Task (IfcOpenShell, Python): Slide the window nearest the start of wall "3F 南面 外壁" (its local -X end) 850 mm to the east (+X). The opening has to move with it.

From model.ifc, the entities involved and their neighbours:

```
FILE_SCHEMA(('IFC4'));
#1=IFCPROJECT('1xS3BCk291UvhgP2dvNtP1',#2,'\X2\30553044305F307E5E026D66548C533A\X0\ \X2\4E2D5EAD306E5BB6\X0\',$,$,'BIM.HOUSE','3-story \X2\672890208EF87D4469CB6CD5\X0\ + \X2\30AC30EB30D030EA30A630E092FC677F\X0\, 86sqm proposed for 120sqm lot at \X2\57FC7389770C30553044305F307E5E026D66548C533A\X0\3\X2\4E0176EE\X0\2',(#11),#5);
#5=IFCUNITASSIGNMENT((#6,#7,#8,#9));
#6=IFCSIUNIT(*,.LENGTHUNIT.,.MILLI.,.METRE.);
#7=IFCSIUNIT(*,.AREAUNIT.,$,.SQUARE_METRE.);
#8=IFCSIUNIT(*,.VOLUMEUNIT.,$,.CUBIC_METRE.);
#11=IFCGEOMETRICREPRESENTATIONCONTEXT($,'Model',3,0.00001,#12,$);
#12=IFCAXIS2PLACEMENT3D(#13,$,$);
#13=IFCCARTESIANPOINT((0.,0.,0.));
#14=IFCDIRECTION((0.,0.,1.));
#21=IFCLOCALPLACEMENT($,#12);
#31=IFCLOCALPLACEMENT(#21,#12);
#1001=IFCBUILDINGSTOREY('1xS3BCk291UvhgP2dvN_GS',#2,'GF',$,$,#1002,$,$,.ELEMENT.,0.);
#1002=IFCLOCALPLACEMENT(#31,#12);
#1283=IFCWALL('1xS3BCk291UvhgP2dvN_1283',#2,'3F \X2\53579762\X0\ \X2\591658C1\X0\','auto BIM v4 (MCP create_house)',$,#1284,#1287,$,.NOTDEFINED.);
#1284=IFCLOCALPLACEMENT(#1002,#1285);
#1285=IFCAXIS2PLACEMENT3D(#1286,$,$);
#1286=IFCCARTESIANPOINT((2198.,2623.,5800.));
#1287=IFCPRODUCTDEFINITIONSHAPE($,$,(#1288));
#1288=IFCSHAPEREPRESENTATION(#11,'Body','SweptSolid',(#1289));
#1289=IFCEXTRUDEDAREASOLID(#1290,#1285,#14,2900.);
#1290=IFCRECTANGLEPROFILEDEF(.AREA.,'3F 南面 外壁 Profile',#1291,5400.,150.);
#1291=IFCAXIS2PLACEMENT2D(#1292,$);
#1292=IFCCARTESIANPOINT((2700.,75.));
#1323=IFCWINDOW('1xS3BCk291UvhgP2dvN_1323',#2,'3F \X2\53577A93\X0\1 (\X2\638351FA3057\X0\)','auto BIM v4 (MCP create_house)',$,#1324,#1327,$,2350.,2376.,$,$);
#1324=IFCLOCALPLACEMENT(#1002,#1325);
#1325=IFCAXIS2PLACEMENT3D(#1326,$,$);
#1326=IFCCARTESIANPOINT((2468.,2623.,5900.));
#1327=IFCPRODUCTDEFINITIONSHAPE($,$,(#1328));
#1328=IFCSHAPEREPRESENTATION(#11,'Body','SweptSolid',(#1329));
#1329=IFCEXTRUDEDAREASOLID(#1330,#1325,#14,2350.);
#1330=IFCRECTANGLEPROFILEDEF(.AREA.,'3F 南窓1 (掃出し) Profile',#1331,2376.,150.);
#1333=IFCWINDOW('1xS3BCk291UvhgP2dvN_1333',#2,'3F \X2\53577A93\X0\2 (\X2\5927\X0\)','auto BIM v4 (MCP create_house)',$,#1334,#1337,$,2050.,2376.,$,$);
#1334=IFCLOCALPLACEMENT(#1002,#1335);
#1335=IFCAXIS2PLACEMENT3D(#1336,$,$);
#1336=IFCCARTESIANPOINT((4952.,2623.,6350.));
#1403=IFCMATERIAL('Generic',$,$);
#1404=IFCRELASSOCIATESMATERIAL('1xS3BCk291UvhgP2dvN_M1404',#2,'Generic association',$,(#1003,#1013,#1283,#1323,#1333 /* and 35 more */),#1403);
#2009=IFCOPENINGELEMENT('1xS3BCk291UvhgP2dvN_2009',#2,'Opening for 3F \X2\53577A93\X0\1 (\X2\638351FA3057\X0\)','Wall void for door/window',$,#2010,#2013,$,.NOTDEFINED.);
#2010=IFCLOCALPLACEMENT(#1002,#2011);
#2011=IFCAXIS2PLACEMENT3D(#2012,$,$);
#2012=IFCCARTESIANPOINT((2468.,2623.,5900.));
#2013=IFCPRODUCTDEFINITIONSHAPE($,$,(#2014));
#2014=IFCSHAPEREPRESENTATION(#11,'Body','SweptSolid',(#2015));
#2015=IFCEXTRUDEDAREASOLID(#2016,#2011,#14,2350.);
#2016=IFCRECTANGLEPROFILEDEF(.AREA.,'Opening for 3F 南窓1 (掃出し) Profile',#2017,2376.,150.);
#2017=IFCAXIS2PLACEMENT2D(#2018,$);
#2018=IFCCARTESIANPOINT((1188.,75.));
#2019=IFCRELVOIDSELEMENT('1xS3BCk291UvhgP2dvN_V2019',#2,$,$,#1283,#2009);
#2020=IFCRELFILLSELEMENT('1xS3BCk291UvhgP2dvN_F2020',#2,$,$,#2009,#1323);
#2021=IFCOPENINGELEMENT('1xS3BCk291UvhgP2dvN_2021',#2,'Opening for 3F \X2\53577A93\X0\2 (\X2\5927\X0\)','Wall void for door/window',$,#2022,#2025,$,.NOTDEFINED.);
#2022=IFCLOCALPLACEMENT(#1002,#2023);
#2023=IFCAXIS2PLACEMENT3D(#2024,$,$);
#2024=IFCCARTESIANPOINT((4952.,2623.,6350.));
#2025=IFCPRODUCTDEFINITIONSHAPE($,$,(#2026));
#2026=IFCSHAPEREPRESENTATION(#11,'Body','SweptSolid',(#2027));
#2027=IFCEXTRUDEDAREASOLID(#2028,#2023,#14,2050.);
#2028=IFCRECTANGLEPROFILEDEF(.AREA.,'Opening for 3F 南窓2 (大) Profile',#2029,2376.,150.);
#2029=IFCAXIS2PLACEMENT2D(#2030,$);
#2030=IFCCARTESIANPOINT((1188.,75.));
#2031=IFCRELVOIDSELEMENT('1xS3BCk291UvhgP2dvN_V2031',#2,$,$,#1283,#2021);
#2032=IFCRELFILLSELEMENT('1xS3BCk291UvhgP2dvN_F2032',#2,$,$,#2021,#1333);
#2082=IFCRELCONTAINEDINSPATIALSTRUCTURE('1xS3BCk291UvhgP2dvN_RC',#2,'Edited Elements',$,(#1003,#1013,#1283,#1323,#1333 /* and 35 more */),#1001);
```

```python
import ifcopenshell
import ifcopenshell.api.geometry
import ifcopenshell.util.placement
import ifcopenshell.util.unit

model = ifcopenshell.open("model.ifc")
unit_scale = ifcopenshell.util.unit.calculate_unit_scale(model)

window = model.by_guid("1xS3BCk291UvhgP2dvN_1323")
opening = window.FillsVoids[0].RelatingOpeningElement
wall = opening.VoidsElements[0].RelatingBuildingElement

wall_matrix = ifcopenshell.util.placement.get_local_placement(wall.ObjectPlacement)
shift = wall_matrix[:3, 0] * 0.85 / unit_scale
before = ifcopenshell.util.placement.get_local_placement(window.ObjectPlacement)[:3, 3].copy()

# The window is not placed relative to its opening, so move both.
for product in (opening, window):
    matrix = ifcopenshell.util.placement.get_local_placement(product.ObjectPlacement)
    matrix[:3, 3] += shift
    ifcopenshell.api.geometry.edit_object_placement(model, product=product, matrix=matrix, is_si=False)

after = ifcopenshell.util.placement.get_local_placement(window.ObjectPlacement)[:3, 3]
print("window moved by", (after - before).round(3) + 0.0)

model.write("model_v2.ifc")
```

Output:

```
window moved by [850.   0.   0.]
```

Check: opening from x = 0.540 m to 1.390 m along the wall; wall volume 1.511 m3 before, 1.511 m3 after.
